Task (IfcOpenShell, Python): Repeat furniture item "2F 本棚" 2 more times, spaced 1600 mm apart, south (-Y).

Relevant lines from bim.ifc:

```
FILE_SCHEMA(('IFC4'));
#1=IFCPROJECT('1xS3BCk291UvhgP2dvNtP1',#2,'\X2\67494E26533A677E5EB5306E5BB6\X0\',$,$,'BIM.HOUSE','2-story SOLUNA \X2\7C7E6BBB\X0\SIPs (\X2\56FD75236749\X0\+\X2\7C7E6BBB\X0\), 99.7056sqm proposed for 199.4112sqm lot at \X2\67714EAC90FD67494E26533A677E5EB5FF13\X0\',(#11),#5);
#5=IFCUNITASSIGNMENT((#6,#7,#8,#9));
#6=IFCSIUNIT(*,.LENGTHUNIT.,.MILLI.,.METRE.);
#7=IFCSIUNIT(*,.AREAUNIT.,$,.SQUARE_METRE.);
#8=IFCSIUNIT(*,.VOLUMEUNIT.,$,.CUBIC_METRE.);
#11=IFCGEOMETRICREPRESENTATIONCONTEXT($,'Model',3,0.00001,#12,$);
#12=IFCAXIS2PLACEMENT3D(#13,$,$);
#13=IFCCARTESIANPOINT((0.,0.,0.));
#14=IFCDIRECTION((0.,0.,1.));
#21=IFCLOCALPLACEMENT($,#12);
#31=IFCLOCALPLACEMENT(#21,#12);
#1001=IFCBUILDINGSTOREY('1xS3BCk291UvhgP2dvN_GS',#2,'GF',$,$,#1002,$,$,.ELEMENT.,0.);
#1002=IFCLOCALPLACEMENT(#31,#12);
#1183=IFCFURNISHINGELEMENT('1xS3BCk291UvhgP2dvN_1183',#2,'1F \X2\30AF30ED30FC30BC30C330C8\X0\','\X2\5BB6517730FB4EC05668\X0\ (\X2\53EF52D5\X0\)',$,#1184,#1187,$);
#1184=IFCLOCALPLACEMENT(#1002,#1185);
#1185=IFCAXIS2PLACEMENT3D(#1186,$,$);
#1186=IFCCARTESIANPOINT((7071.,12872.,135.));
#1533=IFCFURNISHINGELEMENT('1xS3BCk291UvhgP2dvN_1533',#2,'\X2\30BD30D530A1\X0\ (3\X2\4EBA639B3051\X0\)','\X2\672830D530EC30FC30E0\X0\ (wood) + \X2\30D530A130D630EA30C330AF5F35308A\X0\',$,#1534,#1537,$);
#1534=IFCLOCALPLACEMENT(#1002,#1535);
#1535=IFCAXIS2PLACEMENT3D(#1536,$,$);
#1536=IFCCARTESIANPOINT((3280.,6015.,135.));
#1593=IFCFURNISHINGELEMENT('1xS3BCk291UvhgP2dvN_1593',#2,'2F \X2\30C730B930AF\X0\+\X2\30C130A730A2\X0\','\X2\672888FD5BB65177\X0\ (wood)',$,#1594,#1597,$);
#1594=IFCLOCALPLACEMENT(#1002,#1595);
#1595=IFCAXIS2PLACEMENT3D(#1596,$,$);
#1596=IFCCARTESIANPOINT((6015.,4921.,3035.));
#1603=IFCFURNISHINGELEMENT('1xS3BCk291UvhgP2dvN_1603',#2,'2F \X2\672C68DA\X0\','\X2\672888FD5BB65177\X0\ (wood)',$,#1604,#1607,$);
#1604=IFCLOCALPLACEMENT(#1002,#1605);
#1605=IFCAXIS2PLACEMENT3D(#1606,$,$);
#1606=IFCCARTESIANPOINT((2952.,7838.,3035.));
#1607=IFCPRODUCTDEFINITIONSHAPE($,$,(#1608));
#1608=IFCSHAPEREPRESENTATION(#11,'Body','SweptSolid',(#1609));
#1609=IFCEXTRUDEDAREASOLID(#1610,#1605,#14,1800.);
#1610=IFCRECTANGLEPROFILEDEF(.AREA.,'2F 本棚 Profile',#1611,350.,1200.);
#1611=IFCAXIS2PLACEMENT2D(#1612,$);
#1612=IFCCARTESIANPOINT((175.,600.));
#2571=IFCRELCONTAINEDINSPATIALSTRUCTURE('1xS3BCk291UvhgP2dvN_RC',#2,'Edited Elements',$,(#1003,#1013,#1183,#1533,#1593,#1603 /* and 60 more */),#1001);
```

```python
import numpy as np
import ifcopenshell
import ifcopenshell.api.geometry
import ifcopenshell.api.root
import ifcopenshell.util.element
import ifcopenshell.util.placement
import ifcopenshell.util.unit

model = ifcopenshell.open("bim.ifc")
unit_scale = ifcopenshell.util.unit.calculate_unit_scale(model)


def reuse_history(source, copy):
    """copy_class also copies each property set's owner history, people and application; keep the originals."""
    for rel in copy.IsDefinedBy:
        if rel.is_a("IfcRelDefinesByProperties") and (history := rel.RelatingPropertyDefinition.OwnerHistory):
            rel.RelatingPropertyDefinition.OwnerHistory = source.OwnerHistory
            ifcopenshell.util.element.remove_deep2(model, history)


source = model.by_guid("1xS3BCk291UvhgP2dvN_1603")
base = ifcopenshell.util.placement.get_local_placement(source.ObjectPlacement)
step = np.array([0.0, -1.0, 0.0]) * 1.6 / unit_scale

for i in range(1, 3):
    copy = ifcopenshell.api.root.copy_class(model, product=source)
    copy.Representation = ifcopenshell.util.element.copy_deep(
        model, source.Representation, exclude=["IfcGeometricRepresentationContext", "IfcRepresentationMap"]
    )
    reuse_history(source, copy)
    matrix = base.copy()
    matrix[:3, 3] += i * step
    print("added at", matrix[:3, 3].round(3) + 0.0)
    ifcopenshell.api.geometry.edit_object_placement(model, product=copy, matrix=matrix, is_si=False)

model.write("bim_edited.ifc")
```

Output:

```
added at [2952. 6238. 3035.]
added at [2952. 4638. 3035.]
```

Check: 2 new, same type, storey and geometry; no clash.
